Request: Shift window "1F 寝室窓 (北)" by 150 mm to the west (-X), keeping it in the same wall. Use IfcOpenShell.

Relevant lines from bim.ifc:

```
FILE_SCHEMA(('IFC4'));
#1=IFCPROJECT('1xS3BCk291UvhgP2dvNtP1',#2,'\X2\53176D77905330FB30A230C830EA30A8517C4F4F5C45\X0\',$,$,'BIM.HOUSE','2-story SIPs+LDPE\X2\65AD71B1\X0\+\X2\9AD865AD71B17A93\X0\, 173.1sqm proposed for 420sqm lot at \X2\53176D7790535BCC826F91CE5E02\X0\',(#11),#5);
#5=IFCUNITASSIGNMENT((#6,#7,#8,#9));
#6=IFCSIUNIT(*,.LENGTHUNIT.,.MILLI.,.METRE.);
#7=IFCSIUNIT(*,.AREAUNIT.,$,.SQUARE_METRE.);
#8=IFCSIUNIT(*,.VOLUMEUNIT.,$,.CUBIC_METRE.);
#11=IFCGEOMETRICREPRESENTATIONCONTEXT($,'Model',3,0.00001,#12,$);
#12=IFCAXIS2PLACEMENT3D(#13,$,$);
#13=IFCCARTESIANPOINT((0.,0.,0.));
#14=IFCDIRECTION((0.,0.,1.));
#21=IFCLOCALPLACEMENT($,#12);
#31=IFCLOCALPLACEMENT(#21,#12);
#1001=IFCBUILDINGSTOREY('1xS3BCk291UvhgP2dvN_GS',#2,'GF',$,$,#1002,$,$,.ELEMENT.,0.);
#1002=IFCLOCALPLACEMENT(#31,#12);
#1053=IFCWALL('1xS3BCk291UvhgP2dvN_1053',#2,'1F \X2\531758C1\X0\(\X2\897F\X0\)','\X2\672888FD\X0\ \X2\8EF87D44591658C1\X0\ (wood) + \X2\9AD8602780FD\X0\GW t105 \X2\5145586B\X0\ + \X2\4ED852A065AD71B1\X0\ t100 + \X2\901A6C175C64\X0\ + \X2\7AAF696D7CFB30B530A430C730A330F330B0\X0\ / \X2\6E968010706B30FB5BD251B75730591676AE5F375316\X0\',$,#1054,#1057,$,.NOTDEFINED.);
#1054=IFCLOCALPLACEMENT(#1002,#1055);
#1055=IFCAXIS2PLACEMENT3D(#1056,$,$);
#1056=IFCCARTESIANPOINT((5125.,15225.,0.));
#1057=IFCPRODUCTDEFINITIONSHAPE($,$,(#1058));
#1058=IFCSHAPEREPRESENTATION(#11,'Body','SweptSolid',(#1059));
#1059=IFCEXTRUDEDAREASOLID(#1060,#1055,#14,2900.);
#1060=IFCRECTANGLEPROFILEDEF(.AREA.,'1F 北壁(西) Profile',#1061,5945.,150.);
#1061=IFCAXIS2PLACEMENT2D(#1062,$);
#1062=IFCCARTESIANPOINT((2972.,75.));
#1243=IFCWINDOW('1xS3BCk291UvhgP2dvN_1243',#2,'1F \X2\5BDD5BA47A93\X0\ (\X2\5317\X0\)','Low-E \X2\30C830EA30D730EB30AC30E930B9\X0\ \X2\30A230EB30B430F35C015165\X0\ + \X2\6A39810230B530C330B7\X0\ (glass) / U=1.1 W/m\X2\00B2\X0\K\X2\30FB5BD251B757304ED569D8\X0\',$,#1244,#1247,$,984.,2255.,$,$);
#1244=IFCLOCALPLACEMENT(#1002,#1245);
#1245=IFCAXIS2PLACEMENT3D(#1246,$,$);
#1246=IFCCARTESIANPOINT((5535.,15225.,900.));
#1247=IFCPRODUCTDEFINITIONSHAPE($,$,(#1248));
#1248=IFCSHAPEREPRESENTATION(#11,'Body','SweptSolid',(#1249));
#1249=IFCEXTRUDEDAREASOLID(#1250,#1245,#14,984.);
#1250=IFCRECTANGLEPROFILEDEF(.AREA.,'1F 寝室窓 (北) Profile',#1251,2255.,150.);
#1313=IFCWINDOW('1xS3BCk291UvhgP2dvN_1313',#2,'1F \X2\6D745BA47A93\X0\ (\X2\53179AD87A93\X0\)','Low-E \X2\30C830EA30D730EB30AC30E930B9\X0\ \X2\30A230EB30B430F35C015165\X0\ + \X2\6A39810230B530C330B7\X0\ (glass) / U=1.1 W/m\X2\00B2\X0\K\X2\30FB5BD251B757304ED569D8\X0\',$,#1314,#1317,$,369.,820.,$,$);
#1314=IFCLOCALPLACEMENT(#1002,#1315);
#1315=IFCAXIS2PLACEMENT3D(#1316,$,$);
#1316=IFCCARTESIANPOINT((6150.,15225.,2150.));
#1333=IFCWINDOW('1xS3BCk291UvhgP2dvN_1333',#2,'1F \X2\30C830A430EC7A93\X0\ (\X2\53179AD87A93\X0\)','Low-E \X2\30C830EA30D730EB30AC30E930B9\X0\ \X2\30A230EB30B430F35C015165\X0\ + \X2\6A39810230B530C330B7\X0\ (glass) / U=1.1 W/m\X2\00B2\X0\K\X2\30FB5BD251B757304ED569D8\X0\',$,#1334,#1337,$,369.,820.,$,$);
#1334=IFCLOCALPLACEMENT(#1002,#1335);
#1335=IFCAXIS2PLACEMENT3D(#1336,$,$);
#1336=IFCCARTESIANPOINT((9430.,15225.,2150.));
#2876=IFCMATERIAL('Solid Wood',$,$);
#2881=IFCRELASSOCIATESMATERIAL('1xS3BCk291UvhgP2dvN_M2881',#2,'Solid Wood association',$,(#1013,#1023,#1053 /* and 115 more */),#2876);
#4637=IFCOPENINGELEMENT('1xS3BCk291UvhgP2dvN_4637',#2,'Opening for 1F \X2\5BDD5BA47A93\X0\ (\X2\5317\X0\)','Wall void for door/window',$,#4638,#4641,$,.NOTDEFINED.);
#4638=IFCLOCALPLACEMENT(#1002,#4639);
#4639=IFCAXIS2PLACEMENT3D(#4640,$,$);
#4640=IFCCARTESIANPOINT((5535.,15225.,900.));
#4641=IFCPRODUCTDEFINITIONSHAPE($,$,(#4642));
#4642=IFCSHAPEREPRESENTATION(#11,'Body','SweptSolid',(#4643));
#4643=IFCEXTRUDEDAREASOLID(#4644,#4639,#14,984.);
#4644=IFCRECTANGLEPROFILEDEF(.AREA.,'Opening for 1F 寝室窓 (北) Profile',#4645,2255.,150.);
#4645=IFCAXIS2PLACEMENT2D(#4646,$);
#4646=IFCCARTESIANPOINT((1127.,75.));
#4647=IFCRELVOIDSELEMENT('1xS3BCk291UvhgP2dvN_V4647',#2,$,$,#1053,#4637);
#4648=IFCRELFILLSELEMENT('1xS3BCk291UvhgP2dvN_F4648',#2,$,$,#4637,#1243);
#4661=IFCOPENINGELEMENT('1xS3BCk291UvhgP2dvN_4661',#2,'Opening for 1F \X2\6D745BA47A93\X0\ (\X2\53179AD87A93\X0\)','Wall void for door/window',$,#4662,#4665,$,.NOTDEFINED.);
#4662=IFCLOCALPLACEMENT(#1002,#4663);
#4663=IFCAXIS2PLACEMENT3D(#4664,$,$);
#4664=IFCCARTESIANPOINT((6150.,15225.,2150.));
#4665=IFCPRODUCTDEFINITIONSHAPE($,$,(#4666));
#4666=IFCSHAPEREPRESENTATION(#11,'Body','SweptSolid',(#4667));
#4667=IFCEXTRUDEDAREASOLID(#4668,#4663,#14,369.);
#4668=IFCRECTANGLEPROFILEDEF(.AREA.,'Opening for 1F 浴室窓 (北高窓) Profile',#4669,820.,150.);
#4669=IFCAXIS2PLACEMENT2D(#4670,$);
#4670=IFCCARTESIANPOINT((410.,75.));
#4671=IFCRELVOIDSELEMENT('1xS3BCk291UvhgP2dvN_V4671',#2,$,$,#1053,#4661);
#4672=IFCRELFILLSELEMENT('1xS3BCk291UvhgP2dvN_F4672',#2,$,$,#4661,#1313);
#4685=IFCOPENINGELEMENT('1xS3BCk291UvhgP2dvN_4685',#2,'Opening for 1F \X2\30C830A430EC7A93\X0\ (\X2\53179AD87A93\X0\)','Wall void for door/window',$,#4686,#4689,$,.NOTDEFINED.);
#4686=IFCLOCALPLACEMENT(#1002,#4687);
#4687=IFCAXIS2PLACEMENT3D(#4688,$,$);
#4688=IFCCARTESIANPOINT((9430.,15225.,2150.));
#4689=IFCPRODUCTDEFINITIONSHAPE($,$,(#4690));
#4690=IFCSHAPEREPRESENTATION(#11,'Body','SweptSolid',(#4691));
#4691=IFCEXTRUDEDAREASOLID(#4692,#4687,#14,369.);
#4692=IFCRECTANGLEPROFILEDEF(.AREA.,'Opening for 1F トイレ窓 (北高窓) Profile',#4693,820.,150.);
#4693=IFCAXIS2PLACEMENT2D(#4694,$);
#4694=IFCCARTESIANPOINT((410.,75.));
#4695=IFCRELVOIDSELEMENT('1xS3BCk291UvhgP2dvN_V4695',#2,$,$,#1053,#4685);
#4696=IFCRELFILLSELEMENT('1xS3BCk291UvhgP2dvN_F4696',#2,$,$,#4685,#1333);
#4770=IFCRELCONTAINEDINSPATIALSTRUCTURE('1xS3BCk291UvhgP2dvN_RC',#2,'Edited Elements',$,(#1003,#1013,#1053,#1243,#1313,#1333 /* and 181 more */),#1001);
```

```python
import ifcopenshell
import ifcopenshell.api.geometry
import ifcopenshell.util.placement
import ifcopenshell.util.unit

model = ifcopenshell.open("bim.ifc")
unit_scale = ifcopenshell.util.unit.calculate_unit_scale(model)

window = model.by_id(1243)
opening = window.FillsVoids[0].RelatingOpeningElement
wall = opening.VoidsElements[0].RelatingBuildingElement

wall_matrix = ifcopenshell.util.placement.get_local_placement(wall.ObjectPlacement)
shift = wall_matrix[:3, 0] * -0.15 / unit_scale
before = ifcopenshell.util.placement.get_local_placement(window.ObjectPlacement)[:3, 3].copy()

# The window is not placed relative to its opening, so move both.
for product in (opening, window):
    matrix = ifcopenshell.util.placement.get_local_placement(product.ObjectPlacement)
    matrix[:3, 3] += shift
    ifcopenshell.api.geometry.edit_object_placement(model, product=product, matrix=matrix, is_si=False)

after = ifcopenshell.util.placement.get_local_placement(window.ObjectPlacement)[:3, 3]
print("window moved by", (after - before).round(3) + 0.0)

model.write("bim_v2.ifc")
```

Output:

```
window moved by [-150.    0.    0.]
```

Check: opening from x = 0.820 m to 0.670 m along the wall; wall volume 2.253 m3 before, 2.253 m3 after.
